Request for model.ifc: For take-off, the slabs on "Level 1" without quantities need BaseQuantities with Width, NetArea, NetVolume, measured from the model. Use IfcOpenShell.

First a look at what the model holds.

```python
import ifcopenshell
import ifcopenshell.util.element
import ifcopenshell.util.unit

model = ifcopenshell.open("model.ifc")
print(model.schema)
for unit_type in ("LENGTHUNIT", "AREAUNIT", "VOLUMEUNIT"):
    print(unit_type, ifcopenshell.util.unit.calculate_unit_scale(model, unit_type))
storey = next(s for s in model.by_type("IfcBuildingStorey") if s.Name == "Level 1")
slabs = [e for e in ifcopenshell.util.element.get_decomposition(storey) if e.is_a("IfcSlab")]
for e in sorted(slabs, key=lambda e: e.id()):
    print(e.id(), e.is_a(), e.Name, list(ifcopenshell.util.element.get_psets(e, qtos_only=True)), sep=" | ")
```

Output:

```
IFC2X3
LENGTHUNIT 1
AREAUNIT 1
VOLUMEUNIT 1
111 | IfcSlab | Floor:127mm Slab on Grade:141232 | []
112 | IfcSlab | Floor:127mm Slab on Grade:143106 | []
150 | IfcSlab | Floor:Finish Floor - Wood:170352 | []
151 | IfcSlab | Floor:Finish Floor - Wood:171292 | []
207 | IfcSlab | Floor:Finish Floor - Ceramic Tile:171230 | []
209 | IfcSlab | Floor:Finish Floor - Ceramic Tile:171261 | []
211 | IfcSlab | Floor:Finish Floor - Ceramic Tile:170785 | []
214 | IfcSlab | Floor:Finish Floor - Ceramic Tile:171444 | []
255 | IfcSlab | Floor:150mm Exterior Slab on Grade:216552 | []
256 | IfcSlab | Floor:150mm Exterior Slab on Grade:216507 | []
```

```python
import ifcopenshell
import ifcopenshell.api.pset
import ifcopenshell.geom
import ifcopenshell.util.element
import ifcopenshell.util.shape
import ifcopenshell.util.unit

model = ifcopenshell.open("model.ifc")
unit_scale = ifcopenshell.util.unit.calculate_unit_scale(model)
area_scale = ifcopenshell.util.unit.calculate_unit_scale(model, "AREAUNIT")
volume_scale = ifcopenshell.util.unit.calculate_unit_scale(model, "VOLUMEUNIT")
settings = ifcopenshell.geom.settings()

storey = next(s for s in model.by_type("IfcBuildingStorey") if s.Name == "Level 1")
slabs = [e for e in ifcopenshell.util.element.get_decomposition(storey) if e.is_a("IfcSlab")]

for e in sorted(slabs, key=lambda e: e.id()):
    if ifcopenshell.util.element.get_psets(e, qtos_only=True, should_inherit=False):
        continue
    # Geometry comes back in metres, in the element's own axes.
    shape = ifcopenshell.geom.create_shape(settings, e)
    values = {
        "Width": ifcopenshell.util.shape.get_z(shape.geometry) / unit_scale,
        "NetArea": ifcopenshell.util.shape.get_footprint_area(shape.geometry) / area_scale,
        "NetVolume": ifcopenshell.util.shape.get_volume(shape.geometry) / volume_scale,
    }
    qto = ifcopenshell.api.pset.add_qto(model, product=e, name="BaseQuantities")
    ifcopenshell.api.pset.edit_qto(model, qto=qto, properties=values)
    print(e.id(), {k: round(v, 3) for k, v in values.items()})

model.write("model_v2.ifc")
```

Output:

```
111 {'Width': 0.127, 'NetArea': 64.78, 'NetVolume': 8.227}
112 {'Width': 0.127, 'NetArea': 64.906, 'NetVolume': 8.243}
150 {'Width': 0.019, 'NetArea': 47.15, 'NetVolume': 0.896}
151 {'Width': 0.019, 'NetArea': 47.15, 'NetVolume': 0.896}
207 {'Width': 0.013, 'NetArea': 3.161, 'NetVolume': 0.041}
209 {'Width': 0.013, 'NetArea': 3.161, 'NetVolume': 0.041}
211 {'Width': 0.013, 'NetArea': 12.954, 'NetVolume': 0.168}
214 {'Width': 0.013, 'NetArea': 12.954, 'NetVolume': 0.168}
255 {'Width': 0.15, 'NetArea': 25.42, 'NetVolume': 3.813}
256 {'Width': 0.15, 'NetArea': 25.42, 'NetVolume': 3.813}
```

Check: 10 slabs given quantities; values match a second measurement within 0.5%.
